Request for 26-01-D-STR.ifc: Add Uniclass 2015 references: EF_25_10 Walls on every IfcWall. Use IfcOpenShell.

First a look at what the model holds.

```python
import ifcopenshell

model = ifcopenshell.open("26-01-D-STR.ifc")
print(model.schema)
print("classifications:", [c.Name for c in model.by_type("IfcClassification")])
for ifc_class in ("IfcDoor", "IfcRoof", "IfcStair", "IfcWall", "IfcWindow"):
    print(ifc_class, len(model.by_type(ifc_class)))
```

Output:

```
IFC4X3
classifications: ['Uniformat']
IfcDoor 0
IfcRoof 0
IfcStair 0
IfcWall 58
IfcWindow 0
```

```python
import ifcopenshell
import ifcopenshell.api.classification

model = ifcopenshell.open("26-01-D-STR.ifc")

system = ifcopenshell.api.classification.add_classification(model, classification="Uniclass 2015")

codes = {
    "IfcWall": ("EF_25_10", "Walls"),
}
for ifc_class, (code, name) in codes.items():
    products = model.by_type(ifc_class)
    ifcopenshell.api.classification.add_reference(
        model, products=products, classification=system, identification=code, name=name
    )
    print(code, len(products))

model.write("26-01-D-STR_v2.ifc")
```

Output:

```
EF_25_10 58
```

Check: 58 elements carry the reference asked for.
